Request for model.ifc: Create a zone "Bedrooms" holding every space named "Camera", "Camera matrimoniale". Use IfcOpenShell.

First a look at what the model holds.

```python
import ifcopenshell

model = ifcopenshell.open("model.ifc")
print(model.schema)
seen = {}
for space in model.by_type("IfcSpace"):
    seen[space.LongName] = seen.get(space.LongName, 0) + 1
for name, count in sorted(seen.items(), key=str):
    print(count, "x", name)
print("zones:", [z.Name for z in model.by_type("IfcZone")][:20])
```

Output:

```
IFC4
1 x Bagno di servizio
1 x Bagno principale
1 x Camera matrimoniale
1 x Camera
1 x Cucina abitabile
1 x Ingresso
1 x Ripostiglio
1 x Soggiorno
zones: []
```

```python
import ifcopenshell
import ifcopenshell.api.group
import ifcopenshell.api.root

model = ifcopenshell.open("model.ifc")

names = {"Camera", "Camera matrimoniale"}
spaces = [s for s in model.by_type("IfcSpace") if s.LongName in names]

zone = ifcopenshell.api.root.create_entity(model, ifc_class="IfcZone", name="Bedrooms")
ifcopenshell.api.group.assign_group(model, products=spaces, group=zone)
print(len(spaces), "spaces in", zone.Name)

model.write("model_updated.ifc")
```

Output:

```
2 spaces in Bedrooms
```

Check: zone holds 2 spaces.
